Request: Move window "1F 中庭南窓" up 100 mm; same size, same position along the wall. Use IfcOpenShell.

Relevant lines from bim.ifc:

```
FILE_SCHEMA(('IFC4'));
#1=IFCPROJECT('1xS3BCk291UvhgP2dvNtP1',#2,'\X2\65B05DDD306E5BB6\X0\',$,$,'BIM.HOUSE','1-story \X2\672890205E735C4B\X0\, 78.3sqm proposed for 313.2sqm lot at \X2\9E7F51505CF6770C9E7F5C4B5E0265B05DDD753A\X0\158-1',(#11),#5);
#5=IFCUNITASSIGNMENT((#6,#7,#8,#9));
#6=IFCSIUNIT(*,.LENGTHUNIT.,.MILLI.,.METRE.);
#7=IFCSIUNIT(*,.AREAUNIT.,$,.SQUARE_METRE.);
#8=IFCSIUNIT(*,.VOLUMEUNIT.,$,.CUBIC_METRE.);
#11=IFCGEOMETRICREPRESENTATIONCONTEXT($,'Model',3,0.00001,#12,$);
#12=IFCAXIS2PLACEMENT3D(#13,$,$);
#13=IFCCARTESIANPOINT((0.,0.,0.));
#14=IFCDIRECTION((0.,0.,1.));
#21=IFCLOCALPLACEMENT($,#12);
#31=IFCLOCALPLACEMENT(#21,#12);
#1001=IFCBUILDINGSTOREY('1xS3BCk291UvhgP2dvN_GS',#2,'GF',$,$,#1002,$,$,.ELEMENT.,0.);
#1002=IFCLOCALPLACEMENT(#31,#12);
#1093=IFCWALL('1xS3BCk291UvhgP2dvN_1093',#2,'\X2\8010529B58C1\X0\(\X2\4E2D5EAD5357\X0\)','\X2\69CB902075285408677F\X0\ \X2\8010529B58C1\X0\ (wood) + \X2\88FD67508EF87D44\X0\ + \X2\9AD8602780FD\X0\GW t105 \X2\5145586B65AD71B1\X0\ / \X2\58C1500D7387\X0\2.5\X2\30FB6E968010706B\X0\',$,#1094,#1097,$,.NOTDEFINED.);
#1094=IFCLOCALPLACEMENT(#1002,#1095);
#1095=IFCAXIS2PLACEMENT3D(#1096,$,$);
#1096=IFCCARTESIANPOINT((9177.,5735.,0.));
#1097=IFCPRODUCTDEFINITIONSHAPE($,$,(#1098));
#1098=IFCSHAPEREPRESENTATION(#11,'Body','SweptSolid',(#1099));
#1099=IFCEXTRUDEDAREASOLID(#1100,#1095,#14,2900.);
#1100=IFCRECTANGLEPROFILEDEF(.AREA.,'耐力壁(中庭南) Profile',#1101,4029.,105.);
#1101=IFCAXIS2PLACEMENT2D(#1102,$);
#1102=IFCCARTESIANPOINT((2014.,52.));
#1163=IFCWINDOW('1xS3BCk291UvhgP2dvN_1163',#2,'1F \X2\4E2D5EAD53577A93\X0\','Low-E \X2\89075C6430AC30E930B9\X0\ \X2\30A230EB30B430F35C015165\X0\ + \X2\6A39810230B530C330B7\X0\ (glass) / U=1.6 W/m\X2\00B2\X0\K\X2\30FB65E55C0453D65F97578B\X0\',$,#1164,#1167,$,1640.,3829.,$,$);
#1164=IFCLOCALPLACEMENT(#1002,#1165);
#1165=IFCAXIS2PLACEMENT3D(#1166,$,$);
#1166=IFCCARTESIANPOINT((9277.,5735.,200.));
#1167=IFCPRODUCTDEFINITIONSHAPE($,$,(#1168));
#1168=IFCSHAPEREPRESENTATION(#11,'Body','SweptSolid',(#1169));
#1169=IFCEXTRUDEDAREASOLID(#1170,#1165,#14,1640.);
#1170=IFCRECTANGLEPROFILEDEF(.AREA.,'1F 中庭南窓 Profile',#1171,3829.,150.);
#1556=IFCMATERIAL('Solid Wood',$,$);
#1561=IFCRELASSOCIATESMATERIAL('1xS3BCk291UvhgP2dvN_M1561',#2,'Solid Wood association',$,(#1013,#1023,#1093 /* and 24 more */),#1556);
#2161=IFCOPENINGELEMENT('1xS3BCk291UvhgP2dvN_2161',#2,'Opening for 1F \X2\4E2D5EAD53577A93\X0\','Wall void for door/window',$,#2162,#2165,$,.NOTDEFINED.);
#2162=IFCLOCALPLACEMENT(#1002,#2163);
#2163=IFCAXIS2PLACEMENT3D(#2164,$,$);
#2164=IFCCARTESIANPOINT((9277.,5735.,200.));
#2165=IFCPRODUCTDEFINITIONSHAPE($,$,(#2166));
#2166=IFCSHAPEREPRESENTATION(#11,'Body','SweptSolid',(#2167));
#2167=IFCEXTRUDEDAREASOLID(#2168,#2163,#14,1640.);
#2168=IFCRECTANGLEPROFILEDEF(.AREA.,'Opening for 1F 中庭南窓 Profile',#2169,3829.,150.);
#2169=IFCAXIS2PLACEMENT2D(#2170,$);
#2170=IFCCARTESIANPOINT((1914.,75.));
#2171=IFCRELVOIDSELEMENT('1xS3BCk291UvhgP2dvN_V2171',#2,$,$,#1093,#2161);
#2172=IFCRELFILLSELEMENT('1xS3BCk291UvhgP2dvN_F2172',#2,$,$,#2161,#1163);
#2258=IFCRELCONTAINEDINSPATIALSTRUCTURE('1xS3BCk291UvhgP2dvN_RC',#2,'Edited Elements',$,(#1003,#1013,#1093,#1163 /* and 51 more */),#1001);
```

```python
import numpy as np
import ifcopenshell
import ifcopenshell.api.geometry
import ifcopenshell.util.placement
import ifcopenshell.util.unit

model = ifcopenshell.open("bim.ifc")
unit_scale = ifcopenshell.util.unit.calculate_unit_scale(model)

window = model.by_id(1163)
opening = window.FillsVoids[0].RelatingOpeningElement
dz = 100.0

shift = np.array([0.0, 0.0, dz])
# The window is not placed relative to its opening, so move both.
for product in (opening, window):
    matrix = ifcopenshell.util.placement.get_local_placement(product.ObjectPlacement)
    matrix[:3, 3] += shift
    ifcopenshell.api.geometry.edit_object_placement(model, product=product, matrix=matrix, is_si=False)

print(f"moved by {dz * unit_scale:+.3f} m")

model.write("bim_v2.ifc")
```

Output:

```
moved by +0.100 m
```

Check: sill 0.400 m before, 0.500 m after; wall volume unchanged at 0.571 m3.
